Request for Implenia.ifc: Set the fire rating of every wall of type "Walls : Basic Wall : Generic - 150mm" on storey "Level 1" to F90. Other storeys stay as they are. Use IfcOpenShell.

First a look at what the model holds.

```python
import ifcopenshell
import ifcopenshell.util.element

model = ifcopenshell.open("Implenia.ifc")
print(model.schema)
storey = next(s for s in model.by_type("IfcBuildingStorey") if s.Name == "Level 1")
walls = [e for e in ifcopenshell.util.element.get_decomposition(storey) if e.is_a("IfcWall")]
seen = {}
for e in walls:
    element_type = ifcopenshell.util.element.get_type(e)
    key = (element_type.Name if element_type != e and element_type else None, ifcopenshell.util.element.get_pset(e, "Pset_WallCommon", "FireRating"))
    seen[key] = seen.get(key, 0) + 1
for (name, value), count in sorted(seen.items(), key=str):
    print(count, "x", name, "|", value)
```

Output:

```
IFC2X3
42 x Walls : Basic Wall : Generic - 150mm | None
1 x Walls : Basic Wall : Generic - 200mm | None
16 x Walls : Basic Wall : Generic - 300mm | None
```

```python
import ifcopenshell
import ifcopenshell.api.pset
import ifcopenshell.util.element

model = ifcopenshell.open("Implenia.ifc")

storey = next(s for s in model.by_type("IfcBuildingStorey") if s.Name == "Level 1")
walls = [e for e in ifcopenshell.util.element.get_decomposition(storey) if e.is_a("IfcWall")]

count = 0
for e in walls:
    element_type = ifcopenshell.util.element.get_type(e)
    if element_type in (None, e) or element_type.Name != "Walls : Basic Wall : Generic - 150mm":
        continue
    # add_pset returns the element's existing set when there is one.
    pset = ifcopenshell.api.pset.add_pset(model, product=e, name="Pset_WallCommon")
    ifcopenshell.api.pset.edit_pset(model, pset=pset, properties={"FireRating": "F90"})
    count += 1

print(count, "walls updated")

model.write("Implenia_edited.ifc")
```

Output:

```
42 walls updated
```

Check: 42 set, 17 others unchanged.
